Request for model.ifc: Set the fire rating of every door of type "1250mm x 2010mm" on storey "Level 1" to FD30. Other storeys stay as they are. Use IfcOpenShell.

First a look at what the model holds.

```python
import ifcopenshell
import ifcopenshell.util.element

model = ifcopenshell.open("model.ifc")
print(model.schema)
storey = next(s for s in model.by_type("IfcBuildingStorey") if s.Name == "Level 1")
doors = [e for e in ifcopenshell.util.element.get_decomposition(storey) if e.is_a("IfcDoor")]
seen = {}
for e in doors:
    element_type = ifcopenshell.util.element.get_type(e)
    key = (element_type.Name if element_type != e and element_type else None, ifcopenshell.util.element.get_pset(e, "Pset_DoorCommon", "FireRating"))
    seen[key] = seen.get(key, 0) + 1
for (name, value), count in sorted(seen.items(), key=str):
    print(count, "x", name, "|", value)
```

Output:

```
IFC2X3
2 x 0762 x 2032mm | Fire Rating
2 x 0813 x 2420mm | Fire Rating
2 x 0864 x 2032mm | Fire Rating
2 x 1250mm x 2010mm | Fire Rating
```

```python
import ifcopenshell
import ifcopenshell.api.pset
import ifcopenshell.util.element

model = ifcopenshell.open("model.ifc")

storey = next(s for s in model.by_type("IfcBuildingStorey") if s.Name == "Level 1")
doors = [e for e in ifcopenshell.util.element.get_decomposition(storey) if e.is_a("IfcDoor")]

count = 0
for e in doors:
    element_type = ifcopenshell.util.element.get_type(e)
    if element_type in (None, e) or element_type.Name != "1250mm x 2010mm":
        continue
    # add_pset returns the element's existing set when there is one.
    pset = ifcopenshell.api.pset.add_pset(model, product=e, name="Pset_DoorCommon")
    ifcopenshell.api.pset.edit_pset(model, pset=pset, properties={"FireRating": "FD30"})
    count += 1

print(count, "doors updated")

model.write("model_rev.ifc")
```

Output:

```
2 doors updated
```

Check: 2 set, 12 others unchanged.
